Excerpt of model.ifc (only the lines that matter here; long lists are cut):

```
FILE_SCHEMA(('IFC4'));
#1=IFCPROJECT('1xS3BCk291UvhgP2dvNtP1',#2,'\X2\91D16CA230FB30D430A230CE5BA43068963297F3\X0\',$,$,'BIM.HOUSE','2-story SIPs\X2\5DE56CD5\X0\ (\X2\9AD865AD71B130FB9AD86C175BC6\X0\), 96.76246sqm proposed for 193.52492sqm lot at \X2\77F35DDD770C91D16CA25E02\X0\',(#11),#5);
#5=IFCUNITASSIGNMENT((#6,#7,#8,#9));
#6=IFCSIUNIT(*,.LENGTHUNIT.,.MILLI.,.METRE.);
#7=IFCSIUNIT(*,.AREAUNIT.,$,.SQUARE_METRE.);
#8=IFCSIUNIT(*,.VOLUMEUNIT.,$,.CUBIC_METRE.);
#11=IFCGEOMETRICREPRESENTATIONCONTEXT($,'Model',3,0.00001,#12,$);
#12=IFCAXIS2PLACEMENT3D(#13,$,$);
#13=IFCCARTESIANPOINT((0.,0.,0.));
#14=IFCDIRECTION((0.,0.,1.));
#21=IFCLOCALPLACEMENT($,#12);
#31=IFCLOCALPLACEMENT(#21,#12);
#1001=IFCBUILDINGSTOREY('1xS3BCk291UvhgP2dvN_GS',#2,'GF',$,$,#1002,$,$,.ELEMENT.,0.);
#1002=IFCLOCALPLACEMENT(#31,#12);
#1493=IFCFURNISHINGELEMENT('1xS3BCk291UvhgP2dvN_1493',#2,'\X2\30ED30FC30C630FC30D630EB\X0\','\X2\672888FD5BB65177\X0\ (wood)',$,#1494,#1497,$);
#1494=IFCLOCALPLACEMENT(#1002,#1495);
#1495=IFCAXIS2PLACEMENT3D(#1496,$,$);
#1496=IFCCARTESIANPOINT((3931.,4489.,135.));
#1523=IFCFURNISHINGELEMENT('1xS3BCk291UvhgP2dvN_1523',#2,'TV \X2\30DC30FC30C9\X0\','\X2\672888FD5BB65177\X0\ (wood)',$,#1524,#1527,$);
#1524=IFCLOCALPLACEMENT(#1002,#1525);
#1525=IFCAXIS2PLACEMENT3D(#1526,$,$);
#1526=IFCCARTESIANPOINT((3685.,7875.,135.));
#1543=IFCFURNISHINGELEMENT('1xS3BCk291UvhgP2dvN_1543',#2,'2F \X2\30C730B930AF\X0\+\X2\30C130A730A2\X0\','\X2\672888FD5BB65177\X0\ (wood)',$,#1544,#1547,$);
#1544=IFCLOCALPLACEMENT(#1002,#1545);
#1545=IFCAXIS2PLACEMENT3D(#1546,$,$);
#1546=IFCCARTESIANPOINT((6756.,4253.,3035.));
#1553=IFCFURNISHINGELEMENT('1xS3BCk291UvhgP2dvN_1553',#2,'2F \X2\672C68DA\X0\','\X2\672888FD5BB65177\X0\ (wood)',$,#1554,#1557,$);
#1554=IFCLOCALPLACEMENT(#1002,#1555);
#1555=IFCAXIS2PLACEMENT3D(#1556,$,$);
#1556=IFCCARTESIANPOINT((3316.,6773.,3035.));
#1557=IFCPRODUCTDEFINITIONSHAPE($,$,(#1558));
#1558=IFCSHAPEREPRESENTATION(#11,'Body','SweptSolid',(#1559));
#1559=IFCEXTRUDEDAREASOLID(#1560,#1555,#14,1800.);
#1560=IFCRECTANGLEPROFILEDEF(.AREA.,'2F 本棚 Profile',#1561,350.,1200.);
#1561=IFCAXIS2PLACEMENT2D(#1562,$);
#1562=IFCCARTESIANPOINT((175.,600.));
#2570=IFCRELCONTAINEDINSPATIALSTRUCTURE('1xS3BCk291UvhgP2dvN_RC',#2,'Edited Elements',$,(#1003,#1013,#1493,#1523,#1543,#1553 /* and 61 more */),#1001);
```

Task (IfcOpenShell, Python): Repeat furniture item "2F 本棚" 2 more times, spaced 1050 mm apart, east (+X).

```python
import numpy as np
import ifcopenshell
import ifcopenshell.api.geometry
import ifcopenshell.api.root
import ifcopenshell.util.element
import ifcopenshell.util.placement
import ifcopenshell.util.unit

model = ifcopenshell.open("model.ifc")
unit_scale = ifcopenshell.util.unit.calculate_unit_scale(model)


def reuse_history(source, copy):
    """copy_class also copies each property set's owner history, people and application; keep the originals."""
    for rel in copy.IsDefinedBy:
        if rel.is_a("IfcRelDefinesByProperties") and (history := rel.RelatingPropertyDefinition.OwnerHistory):
            rel.RelatingPropertyDefinition.OwnerHistory = source.OwnerHistory
            ifcopenshell.util.element.remove_deep2(model, history)


source = model.by_id(1553)
base = ifcopenshell.util.placement.get_local_placement(source.ObjectPlacement)
step = np.array([1.0, 0.0, 0.0]) * 1.05 / unit_scale

for i in range(1, 3):
    copy = ifcopenshell.api.root.copy_class(model, product=source)
    copy.Representation = ifcopenshell.util.element.copy_deep(
        model, source.Representation, exclude=["IfcGeometricRepresentationContext", "IfcRepresentationMap"]
    )
    reuse_history(source, copy)
    matrix = base.copy()
    matrix[:3, 3] += i * step
    print("added at", matrix[:3, 3].round(3) + 0.0)
    ifcopenshell.api.geometry.edit_object_placement(model, product=copy, matrix=matrix, is_si=False)

model.write("model_edited.ifc")
```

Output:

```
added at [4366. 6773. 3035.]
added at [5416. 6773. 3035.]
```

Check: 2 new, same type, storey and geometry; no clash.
